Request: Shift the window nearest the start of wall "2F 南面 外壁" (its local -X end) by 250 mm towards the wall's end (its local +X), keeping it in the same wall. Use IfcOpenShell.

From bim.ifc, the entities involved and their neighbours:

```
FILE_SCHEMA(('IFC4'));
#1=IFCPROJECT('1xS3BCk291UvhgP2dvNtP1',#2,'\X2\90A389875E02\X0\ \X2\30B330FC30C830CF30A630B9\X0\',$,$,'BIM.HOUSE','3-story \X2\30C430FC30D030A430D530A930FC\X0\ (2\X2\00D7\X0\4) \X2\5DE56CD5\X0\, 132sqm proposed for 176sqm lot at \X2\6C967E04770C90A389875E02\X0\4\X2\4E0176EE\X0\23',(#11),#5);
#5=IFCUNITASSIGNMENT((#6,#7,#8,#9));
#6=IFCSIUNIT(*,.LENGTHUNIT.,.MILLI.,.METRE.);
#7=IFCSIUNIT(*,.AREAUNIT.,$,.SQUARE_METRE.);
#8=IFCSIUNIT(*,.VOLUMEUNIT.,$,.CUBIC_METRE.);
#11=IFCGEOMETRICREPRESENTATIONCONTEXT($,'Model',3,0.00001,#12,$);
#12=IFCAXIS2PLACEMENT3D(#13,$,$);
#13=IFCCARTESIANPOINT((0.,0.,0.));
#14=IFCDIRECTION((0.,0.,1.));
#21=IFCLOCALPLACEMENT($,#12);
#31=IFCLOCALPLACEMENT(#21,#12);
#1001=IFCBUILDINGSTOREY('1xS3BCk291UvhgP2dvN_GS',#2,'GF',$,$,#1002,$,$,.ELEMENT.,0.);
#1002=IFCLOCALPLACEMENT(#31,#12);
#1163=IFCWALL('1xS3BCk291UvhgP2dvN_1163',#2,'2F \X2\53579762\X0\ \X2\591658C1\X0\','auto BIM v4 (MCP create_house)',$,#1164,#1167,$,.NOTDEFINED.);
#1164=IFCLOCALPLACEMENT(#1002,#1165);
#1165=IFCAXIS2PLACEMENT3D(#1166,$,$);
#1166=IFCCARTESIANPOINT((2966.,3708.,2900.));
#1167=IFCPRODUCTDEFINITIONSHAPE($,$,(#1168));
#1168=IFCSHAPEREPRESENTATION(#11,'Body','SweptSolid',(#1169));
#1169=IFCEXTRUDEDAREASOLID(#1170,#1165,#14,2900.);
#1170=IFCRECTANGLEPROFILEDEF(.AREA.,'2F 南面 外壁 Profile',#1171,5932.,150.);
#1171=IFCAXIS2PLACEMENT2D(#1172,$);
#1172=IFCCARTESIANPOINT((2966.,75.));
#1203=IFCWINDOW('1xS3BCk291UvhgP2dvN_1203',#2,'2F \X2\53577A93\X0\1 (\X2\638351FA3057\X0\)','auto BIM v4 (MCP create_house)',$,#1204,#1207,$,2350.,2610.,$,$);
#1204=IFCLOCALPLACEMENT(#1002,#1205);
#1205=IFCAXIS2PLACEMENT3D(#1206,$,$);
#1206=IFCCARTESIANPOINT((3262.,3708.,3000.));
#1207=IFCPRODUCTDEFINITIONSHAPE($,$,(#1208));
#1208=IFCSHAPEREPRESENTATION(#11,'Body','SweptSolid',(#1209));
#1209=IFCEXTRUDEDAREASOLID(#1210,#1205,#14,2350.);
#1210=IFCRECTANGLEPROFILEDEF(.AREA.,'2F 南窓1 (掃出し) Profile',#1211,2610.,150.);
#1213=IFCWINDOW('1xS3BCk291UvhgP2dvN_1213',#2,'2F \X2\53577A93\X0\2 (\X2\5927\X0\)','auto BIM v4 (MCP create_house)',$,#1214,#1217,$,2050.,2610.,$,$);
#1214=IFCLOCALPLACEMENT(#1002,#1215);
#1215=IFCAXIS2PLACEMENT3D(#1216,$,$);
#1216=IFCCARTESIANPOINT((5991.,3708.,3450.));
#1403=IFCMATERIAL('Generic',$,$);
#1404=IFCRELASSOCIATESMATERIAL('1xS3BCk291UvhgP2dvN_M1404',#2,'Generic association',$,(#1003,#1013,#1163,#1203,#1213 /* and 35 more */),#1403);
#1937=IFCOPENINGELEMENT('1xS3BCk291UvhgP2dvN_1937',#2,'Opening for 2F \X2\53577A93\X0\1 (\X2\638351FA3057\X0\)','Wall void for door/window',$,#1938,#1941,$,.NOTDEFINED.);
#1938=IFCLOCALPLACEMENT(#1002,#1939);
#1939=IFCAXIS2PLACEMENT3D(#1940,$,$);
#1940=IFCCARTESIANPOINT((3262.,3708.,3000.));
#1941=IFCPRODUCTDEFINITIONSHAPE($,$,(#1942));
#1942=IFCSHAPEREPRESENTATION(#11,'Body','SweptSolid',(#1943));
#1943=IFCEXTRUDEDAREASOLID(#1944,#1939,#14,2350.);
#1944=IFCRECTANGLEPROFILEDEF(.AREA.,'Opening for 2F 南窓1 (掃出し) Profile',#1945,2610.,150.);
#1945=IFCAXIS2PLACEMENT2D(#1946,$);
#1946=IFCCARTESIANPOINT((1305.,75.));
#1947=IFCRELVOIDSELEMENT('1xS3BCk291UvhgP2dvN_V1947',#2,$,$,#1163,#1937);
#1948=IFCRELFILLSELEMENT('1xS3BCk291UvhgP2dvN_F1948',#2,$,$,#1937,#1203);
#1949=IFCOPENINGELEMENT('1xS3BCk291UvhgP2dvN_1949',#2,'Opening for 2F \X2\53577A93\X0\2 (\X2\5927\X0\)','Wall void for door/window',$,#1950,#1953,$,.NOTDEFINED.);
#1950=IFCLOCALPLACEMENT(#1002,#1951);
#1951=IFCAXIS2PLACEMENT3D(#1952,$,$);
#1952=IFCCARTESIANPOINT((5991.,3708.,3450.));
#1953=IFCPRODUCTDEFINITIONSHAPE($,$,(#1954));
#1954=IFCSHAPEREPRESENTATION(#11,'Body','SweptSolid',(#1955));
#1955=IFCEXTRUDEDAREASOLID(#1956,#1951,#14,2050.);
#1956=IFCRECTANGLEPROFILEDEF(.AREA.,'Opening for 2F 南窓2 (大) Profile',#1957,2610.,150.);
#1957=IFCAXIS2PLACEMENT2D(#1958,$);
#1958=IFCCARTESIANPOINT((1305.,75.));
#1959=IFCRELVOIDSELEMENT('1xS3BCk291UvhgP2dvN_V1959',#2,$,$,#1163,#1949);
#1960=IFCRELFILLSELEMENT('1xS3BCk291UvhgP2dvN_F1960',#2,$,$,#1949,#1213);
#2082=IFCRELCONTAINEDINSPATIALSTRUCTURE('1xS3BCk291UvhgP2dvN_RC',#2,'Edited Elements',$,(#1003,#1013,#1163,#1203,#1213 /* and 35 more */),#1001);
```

```python
import ifcopenshell
import ifcopenshell.api.geometry
import ifcopenshell.util.placement
import ifcopenshell.util.unit

model = ifcopenshell.open("bim.ifc")
unit_scale = ifcopenshell.util.unit.calculate_unit_scale(model)

window = model.by_id(1203)
opening = window.FillsVoids[0].RelatingOpeningElement
wall = opening.VoidsElements[0].RelatingBuildingElement

wall_matrix = ifcopenshell.util.placement.get_local_placement(wall.ObjectPlacement)
shift = wall_matrix[:3, 0] * 0.25 / unit_scale
before = ifcopenshell.util.placement.get_local_placement(window.ObjectPlacement)[:3, 3].copy()

# The window is not placed relative to its opening, so move both.
for product in (opening, window):
    matrix = ifcopenshell.util.placement.get_local_placement(product.ObjectPlacement)
    matrix[:3, 3] += shift
    ifcopenshell.api.geometry.edit_object_placement(model, product=product, matrix=matrix, is_si=False)

after = ifcopenshell.util.placement.get_local_placement(window.ObjectPlacement)[:3, 3]
print("window moved by", (after - before).round(3) + 0.0)

model.write("bim-out.ifc")
```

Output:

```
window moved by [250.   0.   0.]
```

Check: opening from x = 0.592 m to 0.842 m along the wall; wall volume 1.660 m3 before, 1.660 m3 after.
